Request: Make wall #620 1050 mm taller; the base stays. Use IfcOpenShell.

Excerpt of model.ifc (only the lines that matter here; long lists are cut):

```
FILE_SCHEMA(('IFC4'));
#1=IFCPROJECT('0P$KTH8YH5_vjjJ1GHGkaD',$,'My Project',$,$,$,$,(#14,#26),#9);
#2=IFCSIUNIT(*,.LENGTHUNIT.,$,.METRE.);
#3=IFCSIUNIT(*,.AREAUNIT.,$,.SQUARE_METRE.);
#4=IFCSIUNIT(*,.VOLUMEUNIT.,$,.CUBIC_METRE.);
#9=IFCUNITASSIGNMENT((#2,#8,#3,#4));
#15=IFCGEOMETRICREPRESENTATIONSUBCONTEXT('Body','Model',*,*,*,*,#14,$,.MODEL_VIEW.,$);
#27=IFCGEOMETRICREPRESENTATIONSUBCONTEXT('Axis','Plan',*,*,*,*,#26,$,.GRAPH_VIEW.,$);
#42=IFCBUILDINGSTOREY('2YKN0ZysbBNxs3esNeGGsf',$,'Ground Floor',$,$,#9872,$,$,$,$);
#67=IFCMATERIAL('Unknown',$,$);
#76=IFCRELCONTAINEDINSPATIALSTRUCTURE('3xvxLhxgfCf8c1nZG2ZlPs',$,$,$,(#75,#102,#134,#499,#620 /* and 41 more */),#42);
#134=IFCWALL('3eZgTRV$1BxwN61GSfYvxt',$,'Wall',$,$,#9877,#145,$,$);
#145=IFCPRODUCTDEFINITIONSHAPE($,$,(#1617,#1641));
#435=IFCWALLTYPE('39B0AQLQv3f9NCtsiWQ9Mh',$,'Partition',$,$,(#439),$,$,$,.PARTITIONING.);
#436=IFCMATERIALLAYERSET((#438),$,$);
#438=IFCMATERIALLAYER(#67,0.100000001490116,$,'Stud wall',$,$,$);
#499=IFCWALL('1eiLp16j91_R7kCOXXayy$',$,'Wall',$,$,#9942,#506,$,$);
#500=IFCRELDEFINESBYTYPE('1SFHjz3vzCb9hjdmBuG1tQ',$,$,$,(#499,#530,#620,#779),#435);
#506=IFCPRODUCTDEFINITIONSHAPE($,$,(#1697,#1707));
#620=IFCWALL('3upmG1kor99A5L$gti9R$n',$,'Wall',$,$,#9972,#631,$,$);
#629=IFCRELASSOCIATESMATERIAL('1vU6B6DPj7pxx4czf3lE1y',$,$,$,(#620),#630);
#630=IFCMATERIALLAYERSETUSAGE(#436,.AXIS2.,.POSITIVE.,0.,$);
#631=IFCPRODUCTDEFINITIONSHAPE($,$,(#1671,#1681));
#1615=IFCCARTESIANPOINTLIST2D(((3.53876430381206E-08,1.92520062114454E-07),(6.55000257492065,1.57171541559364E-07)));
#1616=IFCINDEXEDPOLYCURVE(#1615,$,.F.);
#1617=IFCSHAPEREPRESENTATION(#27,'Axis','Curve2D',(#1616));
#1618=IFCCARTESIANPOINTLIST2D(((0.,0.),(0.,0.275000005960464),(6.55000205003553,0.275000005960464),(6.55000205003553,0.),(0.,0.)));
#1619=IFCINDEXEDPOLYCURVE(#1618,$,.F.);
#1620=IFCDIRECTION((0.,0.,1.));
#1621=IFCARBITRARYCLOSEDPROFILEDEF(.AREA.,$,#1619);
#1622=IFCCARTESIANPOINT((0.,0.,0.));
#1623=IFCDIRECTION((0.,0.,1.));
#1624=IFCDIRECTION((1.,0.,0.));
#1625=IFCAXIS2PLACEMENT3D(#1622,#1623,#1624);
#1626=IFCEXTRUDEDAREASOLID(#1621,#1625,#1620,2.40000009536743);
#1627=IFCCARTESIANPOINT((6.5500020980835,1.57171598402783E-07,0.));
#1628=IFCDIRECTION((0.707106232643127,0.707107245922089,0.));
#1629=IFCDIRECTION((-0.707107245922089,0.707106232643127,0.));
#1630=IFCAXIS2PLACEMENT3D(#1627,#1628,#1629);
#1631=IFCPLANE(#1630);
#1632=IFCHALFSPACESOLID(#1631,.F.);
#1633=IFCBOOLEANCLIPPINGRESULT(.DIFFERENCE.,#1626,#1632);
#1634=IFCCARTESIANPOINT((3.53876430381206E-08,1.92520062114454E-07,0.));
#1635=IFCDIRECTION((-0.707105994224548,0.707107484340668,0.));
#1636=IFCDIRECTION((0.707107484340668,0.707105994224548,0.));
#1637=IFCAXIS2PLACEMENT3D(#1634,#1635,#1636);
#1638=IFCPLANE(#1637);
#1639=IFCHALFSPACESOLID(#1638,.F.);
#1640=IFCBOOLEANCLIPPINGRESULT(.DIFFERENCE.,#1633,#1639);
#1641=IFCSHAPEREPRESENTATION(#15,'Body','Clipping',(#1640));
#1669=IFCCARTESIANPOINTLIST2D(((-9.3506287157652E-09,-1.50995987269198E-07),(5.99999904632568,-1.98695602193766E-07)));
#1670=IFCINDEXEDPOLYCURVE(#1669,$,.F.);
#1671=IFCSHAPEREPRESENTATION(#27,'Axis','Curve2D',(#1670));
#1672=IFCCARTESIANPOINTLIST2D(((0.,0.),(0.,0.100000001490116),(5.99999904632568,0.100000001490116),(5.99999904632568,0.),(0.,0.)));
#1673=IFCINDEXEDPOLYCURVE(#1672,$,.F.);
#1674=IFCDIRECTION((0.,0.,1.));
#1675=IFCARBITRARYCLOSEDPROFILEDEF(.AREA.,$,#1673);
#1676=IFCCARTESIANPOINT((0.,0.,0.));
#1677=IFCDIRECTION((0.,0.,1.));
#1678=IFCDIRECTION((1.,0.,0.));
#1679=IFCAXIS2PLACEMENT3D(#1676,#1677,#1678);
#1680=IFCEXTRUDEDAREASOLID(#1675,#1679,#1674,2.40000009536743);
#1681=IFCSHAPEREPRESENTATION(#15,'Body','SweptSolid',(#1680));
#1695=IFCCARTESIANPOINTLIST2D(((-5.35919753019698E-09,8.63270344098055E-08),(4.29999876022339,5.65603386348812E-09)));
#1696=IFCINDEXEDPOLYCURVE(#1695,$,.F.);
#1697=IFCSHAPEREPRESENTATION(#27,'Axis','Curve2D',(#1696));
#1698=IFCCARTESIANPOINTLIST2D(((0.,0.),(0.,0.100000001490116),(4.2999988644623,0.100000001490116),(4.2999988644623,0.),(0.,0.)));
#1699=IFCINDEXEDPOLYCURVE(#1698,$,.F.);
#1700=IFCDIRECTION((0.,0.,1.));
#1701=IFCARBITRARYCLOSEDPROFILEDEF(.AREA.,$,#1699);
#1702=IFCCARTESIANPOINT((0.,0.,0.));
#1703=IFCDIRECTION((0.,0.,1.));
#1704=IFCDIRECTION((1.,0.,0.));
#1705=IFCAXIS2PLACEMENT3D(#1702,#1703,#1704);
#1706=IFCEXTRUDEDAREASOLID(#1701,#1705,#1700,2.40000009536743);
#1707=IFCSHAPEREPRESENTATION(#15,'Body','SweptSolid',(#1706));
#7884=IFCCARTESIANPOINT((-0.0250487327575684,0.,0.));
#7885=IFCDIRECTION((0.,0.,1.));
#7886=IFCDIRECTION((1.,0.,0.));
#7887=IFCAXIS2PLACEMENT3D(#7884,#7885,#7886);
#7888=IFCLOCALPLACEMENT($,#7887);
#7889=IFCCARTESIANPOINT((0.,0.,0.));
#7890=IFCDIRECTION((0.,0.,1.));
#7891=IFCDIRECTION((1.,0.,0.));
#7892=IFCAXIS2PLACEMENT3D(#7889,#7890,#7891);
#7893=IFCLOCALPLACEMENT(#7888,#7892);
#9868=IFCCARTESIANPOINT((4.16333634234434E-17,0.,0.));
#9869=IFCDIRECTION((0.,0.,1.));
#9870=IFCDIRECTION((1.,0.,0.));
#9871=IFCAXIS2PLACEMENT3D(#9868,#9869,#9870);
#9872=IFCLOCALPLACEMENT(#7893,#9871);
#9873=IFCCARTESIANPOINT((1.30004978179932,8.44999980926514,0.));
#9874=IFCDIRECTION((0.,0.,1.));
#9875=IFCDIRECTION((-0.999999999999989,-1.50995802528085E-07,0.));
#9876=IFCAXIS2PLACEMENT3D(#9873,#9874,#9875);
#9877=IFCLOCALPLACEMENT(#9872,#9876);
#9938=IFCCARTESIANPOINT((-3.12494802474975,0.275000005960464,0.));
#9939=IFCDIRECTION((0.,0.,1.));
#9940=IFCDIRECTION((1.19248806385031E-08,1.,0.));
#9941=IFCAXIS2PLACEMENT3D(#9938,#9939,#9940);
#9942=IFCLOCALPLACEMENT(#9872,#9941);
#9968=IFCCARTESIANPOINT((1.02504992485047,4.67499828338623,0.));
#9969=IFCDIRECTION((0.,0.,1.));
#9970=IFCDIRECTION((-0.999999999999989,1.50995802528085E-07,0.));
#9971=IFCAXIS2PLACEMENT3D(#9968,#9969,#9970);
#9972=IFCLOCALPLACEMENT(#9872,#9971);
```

```python
import ifcopenshell
import ifcopenshell.geom
import ifcopenshell.util.representation
import ifcopenshell.util.shape
import ifcopenshell.util.unit

model = ifcopenshell.open("model.ifc")
unit_scale = ifcopenshell.util.unit.calculate_unit_scale(model)
settings = ifcopenshell.geom.settings()


def volume(element):
    """Net volume in cubic metres, openings subtracted."""
    shape = ifcopenshell.geom.create_shape(settings, element)
    return ifcopenshell.util.shape.get_volume(shape.geometry)


wall = model.by_guid("3upmG1kor99A5L$gti9R$n")
before = volume(wall)

body = ifcopenshell.util.representation.get_representation(wall, "Model", "Body")
solid = body.Items[0]
old_height = solid.Depth
solid.Depth += 1.05 / unit_scale
after = volume(wall)

print(f"height {old_height:g} -> {solid.Depth:g}, volume {before:.3f} -> {after:.3f} m3")

model.write("model-out.ifc")
```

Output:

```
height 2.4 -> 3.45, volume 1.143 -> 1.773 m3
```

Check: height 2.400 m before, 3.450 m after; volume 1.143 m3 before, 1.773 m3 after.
